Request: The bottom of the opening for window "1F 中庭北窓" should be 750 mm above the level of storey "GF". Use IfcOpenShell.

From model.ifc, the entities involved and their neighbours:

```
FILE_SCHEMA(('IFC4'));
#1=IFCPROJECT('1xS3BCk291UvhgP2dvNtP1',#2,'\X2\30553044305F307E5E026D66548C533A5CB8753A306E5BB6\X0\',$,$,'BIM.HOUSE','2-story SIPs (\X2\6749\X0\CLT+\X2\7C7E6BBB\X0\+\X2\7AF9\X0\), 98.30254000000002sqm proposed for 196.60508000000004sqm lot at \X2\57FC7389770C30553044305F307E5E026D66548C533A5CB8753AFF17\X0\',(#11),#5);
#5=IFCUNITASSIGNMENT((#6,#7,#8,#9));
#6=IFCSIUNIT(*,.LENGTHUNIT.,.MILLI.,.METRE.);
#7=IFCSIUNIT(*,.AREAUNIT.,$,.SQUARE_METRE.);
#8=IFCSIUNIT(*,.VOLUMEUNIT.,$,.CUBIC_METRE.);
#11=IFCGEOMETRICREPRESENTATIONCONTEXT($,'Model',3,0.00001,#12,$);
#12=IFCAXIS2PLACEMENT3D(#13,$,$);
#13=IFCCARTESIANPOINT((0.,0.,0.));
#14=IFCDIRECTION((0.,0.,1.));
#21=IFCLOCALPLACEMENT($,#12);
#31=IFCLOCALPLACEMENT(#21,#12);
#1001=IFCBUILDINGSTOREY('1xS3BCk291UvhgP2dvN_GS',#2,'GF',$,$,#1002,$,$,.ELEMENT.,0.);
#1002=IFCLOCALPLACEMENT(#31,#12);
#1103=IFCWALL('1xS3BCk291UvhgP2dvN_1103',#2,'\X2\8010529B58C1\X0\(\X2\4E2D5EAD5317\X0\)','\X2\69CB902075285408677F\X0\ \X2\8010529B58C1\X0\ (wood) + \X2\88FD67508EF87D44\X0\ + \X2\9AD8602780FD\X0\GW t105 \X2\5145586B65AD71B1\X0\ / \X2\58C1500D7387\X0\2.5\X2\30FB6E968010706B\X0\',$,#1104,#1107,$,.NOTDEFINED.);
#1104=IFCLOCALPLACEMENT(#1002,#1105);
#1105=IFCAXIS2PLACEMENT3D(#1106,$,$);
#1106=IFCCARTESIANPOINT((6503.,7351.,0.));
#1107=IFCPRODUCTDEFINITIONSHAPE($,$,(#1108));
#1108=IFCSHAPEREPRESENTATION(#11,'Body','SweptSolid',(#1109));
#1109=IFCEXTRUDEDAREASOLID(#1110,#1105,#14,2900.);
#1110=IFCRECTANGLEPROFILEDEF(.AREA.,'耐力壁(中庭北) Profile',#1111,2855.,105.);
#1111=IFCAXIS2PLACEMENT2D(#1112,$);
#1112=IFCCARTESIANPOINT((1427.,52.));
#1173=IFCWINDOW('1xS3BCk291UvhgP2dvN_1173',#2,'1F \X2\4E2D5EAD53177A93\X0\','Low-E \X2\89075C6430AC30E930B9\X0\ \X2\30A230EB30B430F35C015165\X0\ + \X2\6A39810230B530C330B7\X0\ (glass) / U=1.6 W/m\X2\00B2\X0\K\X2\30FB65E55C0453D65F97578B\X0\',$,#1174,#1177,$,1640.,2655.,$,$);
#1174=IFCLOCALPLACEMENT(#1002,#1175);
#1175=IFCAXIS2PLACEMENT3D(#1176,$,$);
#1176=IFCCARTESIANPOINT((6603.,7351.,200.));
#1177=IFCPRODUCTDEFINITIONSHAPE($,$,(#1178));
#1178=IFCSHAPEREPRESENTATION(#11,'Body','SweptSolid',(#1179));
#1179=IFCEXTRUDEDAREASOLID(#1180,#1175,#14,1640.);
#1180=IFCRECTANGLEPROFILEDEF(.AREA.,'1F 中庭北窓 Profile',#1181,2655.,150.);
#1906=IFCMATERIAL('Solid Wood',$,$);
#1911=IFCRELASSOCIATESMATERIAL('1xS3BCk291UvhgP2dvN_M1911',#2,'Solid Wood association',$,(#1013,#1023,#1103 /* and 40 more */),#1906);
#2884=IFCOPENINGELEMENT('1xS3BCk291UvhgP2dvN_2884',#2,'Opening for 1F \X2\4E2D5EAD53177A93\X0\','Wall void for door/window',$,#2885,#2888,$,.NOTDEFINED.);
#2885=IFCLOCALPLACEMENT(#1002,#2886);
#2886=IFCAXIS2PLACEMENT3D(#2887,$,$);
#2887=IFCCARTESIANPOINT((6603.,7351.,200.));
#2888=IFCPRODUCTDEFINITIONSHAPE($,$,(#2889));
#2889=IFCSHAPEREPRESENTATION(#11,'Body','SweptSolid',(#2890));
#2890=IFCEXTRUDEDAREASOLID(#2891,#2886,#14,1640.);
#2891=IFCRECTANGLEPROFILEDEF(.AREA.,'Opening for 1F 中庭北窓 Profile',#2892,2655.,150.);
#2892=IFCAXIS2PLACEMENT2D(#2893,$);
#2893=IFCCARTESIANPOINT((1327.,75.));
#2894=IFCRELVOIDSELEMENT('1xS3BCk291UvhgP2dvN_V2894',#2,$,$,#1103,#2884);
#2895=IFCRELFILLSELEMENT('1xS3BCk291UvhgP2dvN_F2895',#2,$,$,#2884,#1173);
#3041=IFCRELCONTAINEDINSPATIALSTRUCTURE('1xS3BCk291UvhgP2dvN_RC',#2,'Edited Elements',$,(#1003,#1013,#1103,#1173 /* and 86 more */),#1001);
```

```python
import numpy as np
import ifcopenshell
import ifcopenshell.api.geometry
import ifcopenshell.geom
import ifcopenshell.util.element
import ifcopenshell.util.placement
import ifcopenshell.util.shape
import ifcopenshell.util.unit

model = ifcopenshell.open("model.ifc")
unit_scale = ifcopenshell.util.unit.calculate_unit_scale(model)

window = model.by_guid("1xS3BCk291UvhgP2dvN_1173")
opening = window.FillsVoids[0].RelatingOpeningElement
storey = ifcopenshell.util.element.get_container(window, ifc_class="IfcBuildingStorey")
level = ifcopenshell.util.placement.get_local_placement(storey.ObjectPlacement)[2, 3]

# The opening's origin need not be at the sill, so measure its lowest point.
shape = ifcopenshell.geom.create_shape(ifcopenshell.geom.settings(), opening)
bottom = ifcopenshell.util.shape.get_shape_bottom_elevation(shape, shape.geometry) / unit_scale
dz = level + 750.0 - bottom

shift = np.array([0.0, 0.0, dz])
# The window is not placed relative to its opening, so move both.
for product in (opening, window):
    matrix = ifcopenshell.util.placement.get_local_placement(product.ObjectPlacement)
    matrix[:3, 3] += shift
    ifcopenshell.api.geometry.edit_object_placement(model, product=product, matrix=matrix, is_si=False)

print(f"moved by {dz * unit_scale:+.3f} m")

model.write("model_updated.ifc")
```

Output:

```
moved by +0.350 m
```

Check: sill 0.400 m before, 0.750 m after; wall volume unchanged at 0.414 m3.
